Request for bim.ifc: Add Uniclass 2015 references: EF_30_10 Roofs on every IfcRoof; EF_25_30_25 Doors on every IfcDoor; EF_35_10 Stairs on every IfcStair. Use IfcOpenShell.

First a look at what the model holds.

```python
import ifcopenshell

model = ifcopenshell.open("bim.ifc")
print(model.schema)
print("classifications:", [c.Name for c in model.by_type("IfcClassification")])
for ifc_class in ("IfcDoor", "IfcRoof", "IfcStair", "IfcWall", "IfcWindow"):
    print(ifc_class, len(model.by_type(ifc_class)))
```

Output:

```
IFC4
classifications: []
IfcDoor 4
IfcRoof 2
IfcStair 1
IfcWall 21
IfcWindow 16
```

```python
import ifcopenshell
import ifcopenshell.api.classification

model = ifcopenshell.open("bim.ifc")

system = ifcopenshell.api.classification.add_classification(model, classification="Uniclass 2015")

codes = {
    "IfcRoof": ("EF_30_10", "Roofs"),
    "IfcDoor": ("EF_25_30_25", "Doors"),
    "IfcStair": ("EF_35_10", "Stairs"),
}
for ifc_class, (code, name) in codes.items():
    products = model.by_type(ifc_class)
    ifcopenshell.api.classification.add_reference(
        model, products=products, classification=system, identification=code, name=name
    )
    print(code, len(products))

model.write("bim_edited.ifc")
```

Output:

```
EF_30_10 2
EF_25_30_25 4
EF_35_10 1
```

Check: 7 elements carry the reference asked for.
